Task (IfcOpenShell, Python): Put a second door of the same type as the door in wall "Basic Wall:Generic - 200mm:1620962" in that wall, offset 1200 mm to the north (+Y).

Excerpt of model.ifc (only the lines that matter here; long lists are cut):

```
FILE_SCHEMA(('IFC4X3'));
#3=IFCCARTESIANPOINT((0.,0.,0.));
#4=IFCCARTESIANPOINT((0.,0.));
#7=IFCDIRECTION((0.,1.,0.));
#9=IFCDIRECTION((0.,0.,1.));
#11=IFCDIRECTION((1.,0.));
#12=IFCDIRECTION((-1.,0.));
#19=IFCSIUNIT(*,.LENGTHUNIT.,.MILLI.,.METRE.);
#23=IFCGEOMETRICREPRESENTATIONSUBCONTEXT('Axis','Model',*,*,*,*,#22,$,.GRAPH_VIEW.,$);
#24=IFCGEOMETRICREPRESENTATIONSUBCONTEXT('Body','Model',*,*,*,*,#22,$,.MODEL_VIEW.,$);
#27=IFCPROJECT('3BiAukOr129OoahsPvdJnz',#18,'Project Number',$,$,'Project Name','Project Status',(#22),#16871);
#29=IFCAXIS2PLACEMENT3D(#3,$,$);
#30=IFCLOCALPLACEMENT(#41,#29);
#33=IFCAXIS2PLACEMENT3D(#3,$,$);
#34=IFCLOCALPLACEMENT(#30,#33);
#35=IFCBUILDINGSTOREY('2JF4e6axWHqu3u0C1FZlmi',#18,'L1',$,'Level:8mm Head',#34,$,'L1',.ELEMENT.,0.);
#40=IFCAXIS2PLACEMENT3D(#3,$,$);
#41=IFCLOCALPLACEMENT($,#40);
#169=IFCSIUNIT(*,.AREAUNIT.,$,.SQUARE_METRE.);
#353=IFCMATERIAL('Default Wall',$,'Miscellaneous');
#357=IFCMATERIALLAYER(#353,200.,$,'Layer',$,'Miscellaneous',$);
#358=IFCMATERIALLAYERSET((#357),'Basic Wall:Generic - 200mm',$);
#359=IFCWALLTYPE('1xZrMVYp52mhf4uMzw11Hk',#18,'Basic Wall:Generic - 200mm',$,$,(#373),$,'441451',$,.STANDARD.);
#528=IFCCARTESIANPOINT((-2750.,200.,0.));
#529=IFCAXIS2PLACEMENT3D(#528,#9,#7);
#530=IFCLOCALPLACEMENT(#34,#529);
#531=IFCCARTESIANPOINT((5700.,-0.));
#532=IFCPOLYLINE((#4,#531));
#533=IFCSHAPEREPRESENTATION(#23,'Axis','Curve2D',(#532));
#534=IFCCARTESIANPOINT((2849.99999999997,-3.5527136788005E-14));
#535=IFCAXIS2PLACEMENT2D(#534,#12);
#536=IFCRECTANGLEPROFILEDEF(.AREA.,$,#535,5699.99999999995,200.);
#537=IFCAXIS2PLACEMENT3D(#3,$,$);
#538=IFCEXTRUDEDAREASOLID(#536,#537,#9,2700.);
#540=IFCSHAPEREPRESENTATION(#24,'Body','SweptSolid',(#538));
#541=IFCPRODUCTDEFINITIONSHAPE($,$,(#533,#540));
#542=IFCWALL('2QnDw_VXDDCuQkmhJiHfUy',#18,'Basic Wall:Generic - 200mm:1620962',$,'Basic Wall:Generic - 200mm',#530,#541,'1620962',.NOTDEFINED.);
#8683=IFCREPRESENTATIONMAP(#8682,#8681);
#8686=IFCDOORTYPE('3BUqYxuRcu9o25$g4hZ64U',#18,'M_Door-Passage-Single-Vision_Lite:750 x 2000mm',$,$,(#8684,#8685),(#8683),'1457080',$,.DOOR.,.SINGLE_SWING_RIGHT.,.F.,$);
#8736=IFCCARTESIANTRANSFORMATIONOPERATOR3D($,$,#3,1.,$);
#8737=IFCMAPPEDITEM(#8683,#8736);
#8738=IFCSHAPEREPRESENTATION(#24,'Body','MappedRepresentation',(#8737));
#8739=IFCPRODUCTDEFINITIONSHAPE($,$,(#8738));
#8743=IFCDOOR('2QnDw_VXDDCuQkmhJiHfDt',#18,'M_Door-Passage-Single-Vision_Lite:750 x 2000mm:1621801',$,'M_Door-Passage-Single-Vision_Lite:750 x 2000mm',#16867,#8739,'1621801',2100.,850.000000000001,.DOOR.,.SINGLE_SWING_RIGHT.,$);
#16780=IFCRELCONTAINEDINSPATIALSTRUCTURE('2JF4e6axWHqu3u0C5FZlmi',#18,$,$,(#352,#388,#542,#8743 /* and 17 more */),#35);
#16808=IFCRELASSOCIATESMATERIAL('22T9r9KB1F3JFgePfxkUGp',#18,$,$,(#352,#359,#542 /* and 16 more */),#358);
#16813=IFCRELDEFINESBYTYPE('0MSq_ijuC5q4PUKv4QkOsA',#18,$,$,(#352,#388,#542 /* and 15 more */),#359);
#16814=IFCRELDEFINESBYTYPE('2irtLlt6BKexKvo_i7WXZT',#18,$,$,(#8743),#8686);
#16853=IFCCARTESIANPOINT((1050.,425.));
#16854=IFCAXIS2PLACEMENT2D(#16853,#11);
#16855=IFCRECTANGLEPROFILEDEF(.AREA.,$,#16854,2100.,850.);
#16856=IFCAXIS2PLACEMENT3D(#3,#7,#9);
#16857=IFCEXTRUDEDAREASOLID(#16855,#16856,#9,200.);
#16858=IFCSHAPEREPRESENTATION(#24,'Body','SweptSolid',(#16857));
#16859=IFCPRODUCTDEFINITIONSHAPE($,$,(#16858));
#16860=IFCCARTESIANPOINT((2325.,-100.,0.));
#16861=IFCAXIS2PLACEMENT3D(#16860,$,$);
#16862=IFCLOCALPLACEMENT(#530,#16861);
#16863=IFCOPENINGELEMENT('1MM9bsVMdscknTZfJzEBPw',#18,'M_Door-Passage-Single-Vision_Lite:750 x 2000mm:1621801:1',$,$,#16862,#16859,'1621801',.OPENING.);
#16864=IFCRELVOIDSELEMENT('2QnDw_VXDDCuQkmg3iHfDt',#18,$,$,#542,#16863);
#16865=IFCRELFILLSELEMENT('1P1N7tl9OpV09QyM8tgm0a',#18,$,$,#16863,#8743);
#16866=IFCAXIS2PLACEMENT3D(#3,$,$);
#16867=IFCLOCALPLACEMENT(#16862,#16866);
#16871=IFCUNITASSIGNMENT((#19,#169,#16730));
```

```python
import ifcopenshell
import ifcopenshell.api.feature
import ifcopenshell.api.geometry
import ifcopenshell.api.root
import ifcopenshell.geom
import ifcopenshell.util.element
import ifcopenshell.util.placement
import ifcopenshell.util.shape
import ifcopenshell.util.unit

model = ifcopenshell.open("model.ifc")
unit_scale = ifcopenshell.util.unit.calculate_unit_scale(model)
settings = ifcopenshell.geom.settings()


def volume(element):
    """Net volume in cubic metres, openings subtracted."""
    shape = ifcopenshell.geom.create_shape(settings, element)
    return ifcopenshell.util.shape.get_volume(shape.geometry)


def reuse_history(source, copy):
    """copy_class also copies each property set's owner history, people and application; keep the originals."""
    for rel in copy.IsDefinedBy:
        if rel.is_a("IfcRelDefinesByProperties") and (history := rel.RelatingPropertyDefinition.OwnerHistory):
            rel.RelatingPropertyDefinition.OwnerHistory = source.OwnerHistory
            ifcopenshell.util.element.remove_deep2(model, history)


door = model.by_guid("2QnDw_VXDDCuQkmhJiHfDt")
opening = door.FillsVoids[0].RelatingOpeningElement
wall = opening.VoidsElements[0].RelatingBuildingElement
before = volume(wall)
shift = ifcopenshell.util.placement.get_local_placement(wall.ObjectPlacement)[:3, 0] * 1.2 / unit_scale

# copy_class copies the void relationship, type, container and properties, but no geometry.
new_opening = ifcopenshell.api.root.copy_class(model, product=opening)
new_opening.Representation = ifcopenshell.util.element.copy_deep(
    model, opening.Representation, exclude=["IfcGeometricRepresentationContext", "IfcRepresentationMap"]
)
new_opening.Name = "M_Door-Passage-Single-Vision_Lite:750 x 2000mm"
new_opening.Tag = None
new_door = ifcopenshell.api.root.copy_class(model, product=door)
new_door.Representation = ifcopenshell.util.element.copy_deep(
    model, door.Representation, exclude=["IfcGeometricRepresentationContext", "IfcRepresentationMap"]
)
new_door.Name = "M_Door-Passage-Single-Vision_Lite:750 x 2000mm"
new_door.Tag = None
reuse_history(door, new_door)
ifcopenshell.api.feature.add_filling(model, opening=new_opening, element=new_door)

for old, new in ((opening, new_opening), (door, new_door)):
    matrix = ifcopenshell.util.placement.get_local_placement(old.ObjectPlacement)
    matrix[:3, 3] += shift
    ifcopenshell.api.geometry.edit_object_placement(model, product=new, matrix=matrix, is_si=False)

after = volume(wall)

print(f"wall volume {before:.3f} -> {after:.3f} m3")

model.write("model_v2.ifc")
```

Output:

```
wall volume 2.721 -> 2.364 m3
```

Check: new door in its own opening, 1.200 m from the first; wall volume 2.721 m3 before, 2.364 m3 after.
